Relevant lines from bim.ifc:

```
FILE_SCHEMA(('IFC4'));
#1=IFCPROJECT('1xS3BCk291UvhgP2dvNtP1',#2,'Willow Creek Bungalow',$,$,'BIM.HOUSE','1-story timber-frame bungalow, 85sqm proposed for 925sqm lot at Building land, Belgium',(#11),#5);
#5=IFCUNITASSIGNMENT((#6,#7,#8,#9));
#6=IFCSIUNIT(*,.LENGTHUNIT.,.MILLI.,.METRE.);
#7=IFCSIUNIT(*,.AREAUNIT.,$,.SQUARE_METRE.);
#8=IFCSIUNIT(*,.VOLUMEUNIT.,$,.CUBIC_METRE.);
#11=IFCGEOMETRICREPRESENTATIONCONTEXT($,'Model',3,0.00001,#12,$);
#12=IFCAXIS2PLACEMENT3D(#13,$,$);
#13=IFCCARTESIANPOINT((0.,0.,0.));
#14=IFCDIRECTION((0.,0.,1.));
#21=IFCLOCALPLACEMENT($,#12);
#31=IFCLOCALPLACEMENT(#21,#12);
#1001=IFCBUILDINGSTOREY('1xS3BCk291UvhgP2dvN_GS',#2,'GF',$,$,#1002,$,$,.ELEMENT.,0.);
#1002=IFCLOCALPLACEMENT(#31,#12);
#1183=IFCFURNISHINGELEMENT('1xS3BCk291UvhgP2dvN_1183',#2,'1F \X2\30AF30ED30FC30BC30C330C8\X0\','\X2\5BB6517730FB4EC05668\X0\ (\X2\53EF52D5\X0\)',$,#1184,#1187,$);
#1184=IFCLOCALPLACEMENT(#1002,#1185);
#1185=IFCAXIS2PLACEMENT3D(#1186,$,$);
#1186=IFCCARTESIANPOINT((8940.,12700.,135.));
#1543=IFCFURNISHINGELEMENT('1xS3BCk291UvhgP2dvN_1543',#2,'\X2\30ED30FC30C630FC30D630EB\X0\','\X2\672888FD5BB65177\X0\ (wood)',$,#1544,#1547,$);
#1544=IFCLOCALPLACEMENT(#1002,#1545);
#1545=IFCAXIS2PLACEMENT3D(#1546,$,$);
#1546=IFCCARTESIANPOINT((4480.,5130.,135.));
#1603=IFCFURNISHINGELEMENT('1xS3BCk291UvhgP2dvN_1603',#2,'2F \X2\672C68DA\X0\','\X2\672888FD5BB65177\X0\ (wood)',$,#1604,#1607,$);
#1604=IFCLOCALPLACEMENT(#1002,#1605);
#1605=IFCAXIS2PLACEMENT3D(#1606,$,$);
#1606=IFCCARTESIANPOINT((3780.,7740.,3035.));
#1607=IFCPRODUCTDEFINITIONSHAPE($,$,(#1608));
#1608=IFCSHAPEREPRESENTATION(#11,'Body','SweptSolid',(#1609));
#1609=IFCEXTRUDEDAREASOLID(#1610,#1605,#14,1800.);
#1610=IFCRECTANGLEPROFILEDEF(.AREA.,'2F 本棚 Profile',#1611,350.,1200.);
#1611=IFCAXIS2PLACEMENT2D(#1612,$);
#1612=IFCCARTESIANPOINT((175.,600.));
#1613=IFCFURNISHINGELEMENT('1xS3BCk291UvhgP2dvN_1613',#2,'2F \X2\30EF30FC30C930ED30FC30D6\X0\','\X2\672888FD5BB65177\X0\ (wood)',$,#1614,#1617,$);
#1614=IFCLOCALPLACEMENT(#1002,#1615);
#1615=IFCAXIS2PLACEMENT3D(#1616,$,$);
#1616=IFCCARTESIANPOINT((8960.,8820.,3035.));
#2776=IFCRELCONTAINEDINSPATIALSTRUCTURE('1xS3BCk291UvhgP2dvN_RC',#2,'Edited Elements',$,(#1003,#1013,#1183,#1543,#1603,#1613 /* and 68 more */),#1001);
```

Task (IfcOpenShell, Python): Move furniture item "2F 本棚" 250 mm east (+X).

```python
import ifcopenshell
import ifcopenshell.api.geometry
import ifcopenshell.util.placement
import ifcopenshell.util.unit

model = ifcopenshell.open("bim.ifc")
unit_scale = ifcopenshell.util.unit.calculate_unit_scale(model)

item = model.by_guid("1xS3BCk291UvhgP2dvN_1603")
matrix = ifcopenshell.util.placement.get_local_placement(item.ObjectPlacement)
matrix[0, 3] += 0.25 / unit_scale
ifcopenshell.api.geometry.edit_object_placement(model, product=item, matrix=matrix, is_si=False)

print(ifcopenshell.util.placement.get_local_placement(item.ObjectPlacement).round(3) + 0.0)

model.write("bim-out.ifc")
```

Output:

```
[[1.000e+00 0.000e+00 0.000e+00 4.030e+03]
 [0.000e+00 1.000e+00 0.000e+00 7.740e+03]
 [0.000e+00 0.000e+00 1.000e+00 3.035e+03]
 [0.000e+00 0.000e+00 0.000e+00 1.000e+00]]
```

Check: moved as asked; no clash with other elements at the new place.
